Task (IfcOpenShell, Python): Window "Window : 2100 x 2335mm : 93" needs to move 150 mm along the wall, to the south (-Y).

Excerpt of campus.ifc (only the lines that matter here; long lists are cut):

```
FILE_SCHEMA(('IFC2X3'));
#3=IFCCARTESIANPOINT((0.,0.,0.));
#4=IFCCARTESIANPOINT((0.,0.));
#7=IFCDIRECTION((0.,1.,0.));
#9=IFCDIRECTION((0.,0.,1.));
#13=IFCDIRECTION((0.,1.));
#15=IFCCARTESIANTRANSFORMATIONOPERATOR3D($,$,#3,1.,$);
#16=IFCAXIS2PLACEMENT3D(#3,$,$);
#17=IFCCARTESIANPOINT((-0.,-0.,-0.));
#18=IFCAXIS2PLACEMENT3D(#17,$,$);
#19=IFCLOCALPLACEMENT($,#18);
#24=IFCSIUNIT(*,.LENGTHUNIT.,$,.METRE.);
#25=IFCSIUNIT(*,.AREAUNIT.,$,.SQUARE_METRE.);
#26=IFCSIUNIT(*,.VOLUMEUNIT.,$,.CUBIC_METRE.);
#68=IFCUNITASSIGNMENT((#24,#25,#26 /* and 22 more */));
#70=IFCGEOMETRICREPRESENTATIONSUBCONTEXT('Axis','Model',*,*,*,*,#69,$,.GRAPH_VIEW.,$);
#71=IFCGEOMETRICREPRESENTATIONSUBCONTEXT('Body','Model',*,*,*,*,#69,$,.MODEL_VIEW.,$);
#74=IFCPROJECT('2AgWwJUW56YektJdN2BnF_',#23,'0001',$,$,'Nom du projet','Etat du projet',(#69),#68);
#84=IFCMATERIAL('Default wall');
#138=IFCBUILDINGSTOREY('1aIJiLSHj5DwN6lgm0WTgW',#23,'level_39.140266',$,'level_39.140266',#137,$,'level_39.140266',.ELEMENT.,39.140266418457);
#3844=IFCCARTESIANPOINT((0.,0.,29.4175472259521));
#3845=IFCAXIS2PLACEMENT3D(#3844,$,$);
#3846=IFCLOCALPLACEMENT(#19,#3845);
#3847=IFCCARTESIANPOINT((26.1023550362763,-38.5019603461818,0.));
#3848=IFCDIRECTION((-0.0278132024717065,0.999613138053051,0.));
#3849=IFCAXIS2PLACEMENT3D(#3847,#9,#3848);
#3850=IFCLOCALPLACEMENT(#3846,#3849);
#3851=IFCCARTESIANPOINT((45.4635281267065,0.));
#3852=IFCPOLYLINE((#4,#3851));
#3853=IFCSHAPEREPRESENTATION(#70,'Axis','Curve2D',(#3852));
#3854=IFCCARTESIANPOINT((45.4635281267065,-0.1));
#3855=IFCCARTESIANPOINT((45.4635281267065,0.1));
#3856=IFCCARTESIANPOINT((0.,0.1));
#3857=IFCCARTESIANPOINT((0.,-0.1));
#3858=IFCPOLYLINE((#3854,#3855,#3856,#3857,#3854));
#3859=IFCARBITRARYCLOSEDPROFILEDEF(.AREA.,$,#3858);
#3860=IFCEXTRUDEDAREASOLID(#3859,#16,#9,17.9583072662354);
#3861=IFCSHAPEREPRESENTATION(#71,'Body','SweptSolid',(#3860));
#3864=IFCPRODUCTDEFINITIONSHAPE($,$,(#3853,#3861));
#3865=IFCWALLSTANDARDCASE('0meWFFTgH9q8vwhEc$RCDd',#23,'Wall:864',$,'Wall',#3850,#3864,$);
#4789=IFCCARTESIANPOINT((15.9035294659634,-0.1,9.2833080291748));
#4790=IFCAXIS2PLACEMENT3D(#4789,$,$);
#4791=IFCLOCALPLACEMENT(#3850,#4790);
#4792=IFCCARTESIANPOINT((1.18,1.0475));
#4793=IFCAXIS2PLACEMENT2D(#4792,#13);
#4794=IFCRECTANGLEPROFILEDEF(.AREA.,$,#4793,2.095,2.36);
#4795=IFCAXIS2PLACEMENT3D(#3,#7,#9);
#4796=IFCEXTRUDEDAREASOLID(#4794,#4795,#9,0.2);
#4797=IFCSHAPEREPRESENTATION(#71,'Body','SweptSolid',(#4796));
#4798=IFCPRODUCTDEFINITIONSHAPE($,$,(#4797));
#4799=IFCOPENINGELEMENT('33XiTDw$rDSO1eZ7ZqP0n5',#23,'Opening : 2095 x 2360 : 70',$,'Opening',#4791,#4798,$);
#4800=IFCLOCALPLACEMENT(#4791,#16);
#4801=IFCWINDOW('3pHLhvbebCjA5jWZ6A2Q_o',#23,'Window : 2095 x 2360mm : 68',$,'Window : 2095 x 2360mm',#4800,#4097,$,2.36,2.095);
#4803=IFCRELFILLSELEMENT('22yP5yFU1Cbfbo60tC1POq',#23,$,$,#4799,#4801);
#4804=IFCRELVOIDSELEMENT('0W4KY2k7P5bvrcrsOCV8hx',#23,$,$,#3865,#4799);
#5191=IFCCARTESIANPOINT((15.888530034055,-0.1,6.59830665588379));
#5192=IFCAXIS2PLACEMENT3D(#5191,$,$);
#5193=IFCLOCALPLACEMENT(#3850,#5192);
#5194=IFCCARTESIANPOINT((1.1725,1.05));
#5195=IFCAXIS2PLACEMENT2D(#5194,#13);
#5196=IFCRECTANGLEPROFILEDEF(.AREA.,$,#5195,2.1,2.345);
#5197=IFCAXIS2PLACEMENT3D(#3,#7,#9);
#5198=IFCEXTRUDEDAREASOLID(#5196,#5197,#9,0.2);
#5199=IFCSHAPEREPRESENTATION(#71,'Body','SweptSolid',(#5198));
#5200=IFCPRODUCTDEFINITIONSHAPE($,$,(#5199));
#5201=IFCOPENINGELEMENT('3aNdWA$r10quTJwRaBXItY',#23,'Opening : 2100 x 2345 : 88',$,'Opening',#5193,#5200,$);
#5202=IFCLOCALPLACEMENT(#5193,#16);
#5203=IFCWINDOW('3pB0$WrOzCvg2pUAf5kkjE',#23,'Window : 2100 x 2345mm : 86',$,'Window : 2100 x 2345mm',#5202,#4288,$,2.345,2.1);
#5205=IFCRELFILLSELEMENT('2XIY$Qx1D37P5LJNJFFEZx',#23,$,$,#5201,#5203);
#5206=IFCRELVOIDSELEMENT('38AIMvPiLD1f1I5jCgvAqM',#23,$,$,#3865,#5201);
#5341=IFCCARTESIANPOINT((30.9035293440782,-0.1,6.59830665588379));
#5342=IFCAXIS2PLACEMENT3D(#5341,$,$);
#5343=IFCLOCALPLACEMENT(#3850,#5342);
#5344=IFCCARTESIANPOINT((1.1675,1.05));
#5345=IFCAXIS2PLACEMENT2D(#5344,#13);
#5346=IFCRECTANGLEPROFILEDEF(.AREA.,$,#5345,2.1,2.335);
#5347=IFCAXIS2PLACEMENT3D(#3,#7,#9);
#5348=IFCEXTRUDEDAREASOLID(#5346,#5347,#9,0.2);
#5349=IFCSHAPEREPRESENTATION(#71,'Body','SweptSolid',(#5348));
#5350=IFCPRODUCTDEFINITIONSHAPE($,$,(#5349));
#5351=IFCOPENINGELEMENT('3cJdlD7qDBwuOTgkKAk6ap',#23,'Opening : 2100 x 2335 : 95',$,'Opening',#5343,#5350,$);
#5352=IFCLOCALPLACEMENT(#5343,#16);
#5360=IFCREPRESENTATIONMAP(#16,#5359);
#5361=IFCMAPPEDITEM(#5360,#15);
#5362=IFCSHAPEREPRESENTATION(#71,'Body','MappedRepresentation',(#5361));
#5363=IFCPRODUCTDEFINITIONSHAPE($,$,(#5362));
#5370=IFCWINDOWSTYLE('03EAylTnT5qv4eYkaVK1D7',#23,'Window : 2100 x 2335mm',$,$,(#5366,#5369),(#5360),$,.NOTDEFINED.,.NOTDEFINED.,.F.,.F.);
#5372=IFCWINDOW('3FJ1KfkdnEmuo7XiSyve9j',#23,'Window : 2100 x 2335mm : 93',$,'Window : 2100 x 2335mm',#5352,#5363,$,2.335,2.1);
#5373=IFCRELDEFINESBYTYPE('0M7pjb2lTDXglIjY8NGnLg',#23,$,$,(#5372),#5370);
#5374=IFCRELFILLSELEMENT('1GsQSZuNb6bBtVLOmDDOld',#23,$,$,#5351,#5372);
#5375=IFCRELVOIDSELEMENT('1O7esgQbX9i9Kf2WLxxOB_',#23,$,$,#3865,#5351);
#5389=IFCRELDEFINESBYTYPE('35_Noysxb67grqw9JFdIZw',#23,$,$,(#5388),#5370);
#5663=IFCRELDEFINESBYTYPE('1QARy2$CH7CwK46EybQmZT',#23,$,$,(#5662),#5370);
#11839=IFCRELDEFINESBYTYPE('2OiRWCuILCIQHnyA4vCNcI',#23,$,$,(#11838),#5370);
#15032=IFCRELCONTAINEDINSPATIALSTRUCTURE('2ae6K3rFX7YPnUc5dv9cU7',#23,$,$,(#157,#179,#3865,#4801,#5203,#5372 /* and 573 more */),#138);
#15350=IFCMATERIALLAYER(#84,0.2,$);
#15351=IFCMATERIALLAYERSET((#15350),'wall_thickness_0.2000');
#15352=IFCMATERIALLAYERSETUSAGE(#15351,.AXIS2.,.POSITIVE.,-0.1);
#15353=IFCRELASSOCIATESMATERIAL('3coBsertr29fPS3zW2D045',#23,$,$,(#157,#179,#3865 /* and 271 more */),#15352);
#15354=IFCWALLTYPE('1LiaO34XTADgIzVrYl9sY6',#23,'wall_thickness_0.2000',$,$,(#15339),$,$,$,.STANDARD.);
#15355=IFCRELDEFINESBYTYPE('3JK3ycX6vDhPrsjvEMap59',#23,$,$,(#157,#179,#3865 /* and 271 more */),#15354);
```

```python
import ifcopenshell
import ifcopenshell.api.geometry
import ifcopenshell.util.placement

model = ifcopenshell.open("campus.ifc")

window = model.by_guid("3FJ1KfkdnEmuo7XiSyve9j")
opening = window.FillsVoids[0].RelatingOpeningElement
wall = opening.VoidsElements[0].RelatingBuildingElement

wall_matrix = ifcopenshell.util.placement.get_local_placement(wall.ObjectPlacement)
shift = wall_matrix[:3, 0] * -0.15
before = ifcopenshell.util.placement.get_local_placement(window.ObjectPlacement)[:3, 3].copy()

# The window is placed relative to its opening, so it follows when the opening moves.
matrix = ifcopenshell.util.placement.get_local_placement(opening.ObjectPlacement)
matrix[:3, 3] += shift
ifcopenshell.api.geometry.edit_object_placement(
    model, product=opening, matrix=matrix, is_si=False, should_transform_children=True
)

after = ifcopenshell.util.placement.get_local_placement(window.ObjectPlacement)[:3, 3]
print("window moved by", (after - before).round(3) + 0.0)

model.write("campus-out.ifc")
```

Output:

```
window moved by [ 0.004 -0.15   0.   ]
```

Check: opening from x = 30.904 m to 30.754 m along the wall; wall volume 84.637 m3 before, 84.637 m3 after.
